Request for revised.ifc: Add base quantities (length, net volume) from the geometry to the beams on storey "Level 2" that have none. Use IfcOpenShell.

First a look at what the model holds.

```python
import ifcopenshell
import ifcopenshell.util.element
import ifcopenshell.util.unit

model = ifcopenshell.open("revised.ifc")
print(model.schema)
for unit_type in ("LENGTHUNIT", "AREAUNIT", "VOLUMEUNIT"):
    print(unit_type, ifcopenshell.util.unit.calculate_unit_scale(model, unit_type))
storey = next(s for s in model.by_type("IfcBuildingStorey") if s.Name == "Level 2")
beams = [e for e in ifcopenshell.util.element.get_decomposition(storey) if e.is_a("IfcBeam")]
for e in sorted(beams, key=lambda e: e.id()):
    print(e.id(), e.is_a(), e.Name, list(ifcopenshell.util.element.get_psets(e, qtos_only=True)), sep=" | ")
```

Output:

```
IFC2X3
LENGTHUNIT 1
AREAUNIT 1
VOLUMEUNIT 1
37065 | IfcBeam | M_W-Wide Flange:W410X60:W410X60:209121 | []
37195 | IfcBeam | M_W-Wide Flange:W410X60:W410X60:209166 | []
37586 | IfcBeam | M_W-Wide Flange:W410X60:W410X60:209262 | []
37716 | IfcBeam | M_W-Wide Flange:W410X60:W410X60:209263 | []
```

```python
import ifcopenshell
import ifcopenshell.api.pset
import ifcopenshell.geom
import ifcopenshell.util.element
import ifcopenshell.util.shape
import ifcopenshell.util.unit

model = ifcopenshell.open("revised.ifc")
unit_scale = ifcopenshell.util.unit.calculate_unit_scale(model)
volume_scale = ifcopenshell.util.unit.calculate_unit_scale(model, "VOLUMEUNIT")
settings = ifcopenshell.geom.settings()

storey = next(s for s in model.by_type("IfcBuildingStorey") if s.Name == "Level 2")
beams = [e for e in ifcopenshell.util.element.get_decomposition(storey) if e.is_a("IfcBeam")]

for e in sorted(beams, key=lambda e: e.id()):
    if ifcopenshell.util.element.get_psets(e, qtos_only=True, should_inherit=False):
        continue
    # Geometry comes back in metres, in the element's own axes.
    shape = ifcopenshell.geom.create_shape(settings, e)
    values = {
        "Length": ifcopenshell.util.shape.get_max_xyz(shape.geometry) / unit_scale,
        "NetVolume": ifcopenshell.util.shape.get_volume(shape.geometry) / volume_scale,
    }
    qto = ifcopenshell.api.pset.add_qto(model, product=e, name="BaseQuantities")
    ifcopenshell.api.pset.edit_qto(model, qto=qto, properties=values)
    print(e.id(), {k: round(v, 3) for k, v in values.items()})

model.write("revised_edited.ifc")
```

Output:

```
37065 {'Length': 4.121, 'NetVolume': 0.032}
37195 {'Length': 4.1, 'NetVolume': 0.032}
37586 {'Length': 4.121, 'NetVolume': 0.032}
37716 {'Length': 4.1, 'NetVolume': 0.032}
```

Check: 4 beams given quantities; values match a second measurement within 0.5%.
